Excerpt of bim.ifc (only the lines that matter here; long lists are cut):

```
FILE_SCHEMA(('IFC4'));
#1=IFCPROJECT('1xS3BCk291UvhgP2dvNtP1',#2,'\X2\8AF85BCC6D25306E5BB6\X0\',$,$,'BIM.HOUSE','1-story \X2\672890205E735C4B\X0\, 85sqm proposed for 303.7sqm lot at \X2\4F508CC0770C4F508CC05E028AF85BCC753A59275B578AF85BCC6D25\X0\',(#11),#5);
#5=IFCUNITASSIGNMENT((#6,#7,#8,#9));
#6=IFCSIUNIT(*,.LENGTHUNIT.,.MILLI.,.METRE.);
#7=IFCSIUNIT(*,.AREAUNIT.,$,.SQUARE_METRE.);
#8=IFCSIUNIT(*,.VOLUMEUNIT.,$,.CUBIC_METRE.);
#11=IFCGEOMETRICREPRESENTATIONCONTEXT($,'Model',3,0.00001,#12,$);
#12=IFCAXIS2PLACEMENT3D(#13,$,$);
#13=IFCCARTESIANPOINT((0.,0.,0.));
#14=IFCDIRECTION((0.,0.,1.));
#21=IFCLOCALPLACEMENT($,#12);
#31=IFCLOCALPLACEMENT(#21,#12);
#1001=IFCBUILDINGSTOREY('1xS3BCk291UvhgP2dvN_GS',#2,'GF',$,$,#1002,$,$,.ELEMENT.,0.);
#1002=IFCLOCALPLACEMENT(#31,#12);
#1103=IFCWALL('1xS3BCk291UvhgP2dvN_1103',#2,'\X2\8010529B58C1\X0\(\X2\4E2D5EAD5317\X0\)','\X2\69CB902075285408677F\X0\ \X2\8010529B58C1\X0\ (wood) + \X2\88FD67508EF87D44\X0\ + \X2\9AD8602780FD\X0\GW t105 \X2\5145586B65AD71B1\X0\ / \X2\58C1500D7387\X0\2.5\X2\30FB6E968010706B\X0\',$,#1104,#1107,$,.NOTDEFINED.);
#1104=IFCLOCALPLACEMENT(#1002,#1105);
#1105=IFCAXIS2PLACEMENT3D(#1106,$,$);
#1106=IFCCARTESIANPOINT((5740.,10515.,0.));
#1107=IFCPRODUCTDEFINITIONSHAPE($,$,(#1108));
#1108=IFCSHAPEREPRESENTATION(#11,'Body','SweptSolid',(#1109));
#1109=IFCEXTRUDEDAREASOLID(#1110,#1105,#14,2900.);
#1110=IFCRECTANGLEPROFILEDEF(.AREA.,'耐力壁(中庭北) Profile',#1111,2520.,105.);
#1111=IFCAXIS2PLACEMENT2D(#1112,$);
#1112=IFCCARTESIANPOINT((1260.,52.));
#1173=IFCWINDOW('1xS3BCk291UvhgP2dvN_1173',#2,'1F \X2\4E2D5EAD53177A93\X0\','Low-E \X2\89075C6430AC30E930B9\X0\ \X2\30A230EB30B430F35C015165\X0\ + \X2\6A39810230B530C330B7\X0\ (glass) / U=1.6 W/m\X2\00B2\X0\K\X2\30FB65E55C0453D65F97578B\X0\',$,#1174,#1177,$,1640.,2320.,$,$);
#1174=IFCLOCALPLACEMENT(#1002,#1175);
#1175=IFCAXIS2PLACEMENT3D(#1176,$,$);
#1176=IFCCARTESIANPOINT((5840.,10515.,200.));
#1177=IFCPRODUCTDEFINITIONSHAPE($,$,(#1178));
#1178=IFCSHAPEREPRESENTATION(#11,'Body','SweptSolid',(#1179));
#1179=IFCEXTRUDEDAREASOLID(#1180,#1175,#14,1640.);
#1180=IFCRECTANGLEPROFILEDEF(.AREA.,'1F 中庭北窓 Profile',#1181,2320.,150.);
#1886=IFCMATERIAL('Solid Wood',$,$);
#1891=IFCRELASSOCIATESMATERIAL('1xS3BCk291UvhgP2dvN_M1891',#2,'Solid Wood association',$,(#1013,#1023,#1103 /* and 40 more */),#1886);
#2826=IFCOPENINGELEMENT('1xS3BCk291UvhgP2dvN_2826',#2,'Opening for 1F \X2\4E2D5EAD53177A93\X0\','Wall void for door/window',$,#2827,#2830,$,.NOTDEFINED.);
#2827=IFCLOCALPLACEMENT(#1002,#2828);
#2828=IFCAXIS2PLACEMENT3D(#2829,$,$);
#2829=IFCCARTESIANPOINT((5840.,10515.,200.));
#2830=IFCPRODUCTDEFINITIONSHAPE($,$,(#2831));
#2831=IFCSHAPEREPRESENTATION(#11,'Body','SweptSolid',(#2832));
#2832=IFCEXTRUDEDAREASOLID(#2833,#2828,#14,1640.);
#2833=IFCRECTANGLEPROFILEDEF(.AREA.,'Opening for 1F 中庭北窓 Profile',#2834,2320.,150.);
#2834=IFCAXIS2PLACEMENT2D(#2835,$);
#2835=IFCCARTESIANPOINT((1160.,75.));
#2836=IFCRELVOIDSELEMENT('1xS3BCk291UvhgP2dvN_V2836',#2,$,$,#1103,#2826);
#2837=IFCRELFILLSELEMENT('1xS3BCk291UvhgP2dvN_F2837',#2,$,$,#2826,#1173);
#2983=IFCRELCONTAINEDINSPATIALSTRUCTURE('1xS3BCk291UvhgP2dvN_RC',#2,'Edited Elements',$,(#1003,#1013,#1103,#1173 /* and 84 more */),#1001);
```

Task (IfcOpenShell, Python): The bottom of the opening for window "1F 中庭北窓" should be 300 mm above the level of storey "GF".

```python
import numpy as np
import ifcopenshell
import ifcopenshell.api.geometry
import ifcopenshell.geom
import ifcopenshell.util.element
import ifcopenshell.util.placement
import ifcopenshell.util.shape
import ifcopenshell.util.unit

model = ifcopenshell.open("bim.ifc")
unit_scale = ifcopenshell.util.unit.calculate_unit_scale(model)

window = model.by_guid("1xS3BCk291UvhgP2dvN_1173")
opening = window.FillsVoids[0].RelatingOpeningElement
storey = ifcopenshell.util.element.get_container(window, ifc_class="IfcBuildingStorey")
level = ifcopenshell.util.placement.get_local_placement(storey.ObjectPlacement)[2, 3]

# The opening's origin need not be at the sill, so measure its lowest point.
shape = ifcopenshell.geom.create_shape(ifcopenshell.geom.settings(), opening)
bottom = ifcopenshell.util.shape.get_shape_bottom_elevation(shape, shape.geometry) / unit_scale
dz = level + 0.3 / unit_scale - bottom

shift = np.array([0.0, 0.0, dz])
# The window is not placed relative to its opening, so move both.
for product in (opening, window):
    matrix = ifcopenshell.util.placement.get_local_placement(product.ObjectPlacement)
    matrix[:3, 3] += shift
    ifcopenshell.api.geometry.edit_object_placement(model, product=product, matrix=matrix, is_si=False)

print(f"moved by {dz * unit_scale:+.3f} m")

model.write("bim-out.ifc")
```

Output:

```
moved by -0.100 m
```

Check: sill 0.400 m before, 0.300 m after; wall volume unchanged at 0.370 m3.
